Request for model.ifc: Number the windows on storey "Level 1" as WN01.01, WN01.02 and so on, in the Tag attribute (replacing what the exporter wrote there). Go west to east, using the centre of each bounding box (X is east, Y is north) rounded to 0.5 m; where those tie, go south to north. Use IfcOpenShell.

First a look at what the model holds.

```python
import ifcopenshell
import ifcopenshell.util.element
import ifcopenshell.util.placement

model = ifcopenshell.open("model.ifc")
print(model.schema)
storey = next(s for s in model.by_type("IfcBuildingStorey") if s.Name == "Level 1")
windows = [e for e in ifcopenshell.util.element.get_decomposition(storey) if e.is_a("IfcWindow")]
for e in sorted(windows, key=lambda e: e.id()):
    origin = ifcopenshell.util.placement.get_local_placement(e.ObjectPlacement)[:3, 3]
    print(e.id(), e.Tag, e.Name, origin.round(2) + 0.0, sep=" | ")
```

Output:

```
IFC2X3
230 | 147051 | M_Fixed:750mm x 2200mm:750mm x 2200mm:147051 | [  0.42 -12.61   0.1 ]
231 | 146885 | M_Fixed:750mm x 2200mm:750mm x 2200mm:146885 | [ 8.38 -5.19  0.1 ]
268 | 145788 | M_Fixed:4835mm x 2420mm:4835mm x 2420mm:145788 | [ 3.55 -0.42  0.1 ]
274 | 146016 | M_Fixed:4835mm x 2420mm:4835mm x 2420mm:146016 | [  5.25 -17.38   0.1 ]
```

```python
import ifcopenshell
import ifcopenshell.geom
import ifcopenshell.util.element
import ifcopenshell.util.shape

model = ifcopenshell.open("model.ifc")
settings = ifcopenshell.geom.settings()
settings.set("use-world-coords", True)


def centre(element):
    shape = ifcopenshell.geom.create_shape(settings, element)
    return ifcopenshell.util.shape.get_bbox_centroid(shape.geometry)


storey = next(s for s in model.by_type("IfcBuildingStorey") if s.Name == "Level 1")
windows = [e for e in ifcopenshell.util.element.get_decomposition(storey) if e.is_a("IfcWindow")]

# Insertion points can sit at a corner or the storey origin, so sort by the geometry (in metres).
centres = {e: centre(e) for e in windows}
windows.sort(key=lambda e: (round(centres[e][0] / 0.5), centres[e][1]))

for i, e in enumerate(windows, start=1):
    number = f"WN01.{i:02d}"
    e.Tag = number
    print(e.id(), number)

model.write("model_edited.ifc")
```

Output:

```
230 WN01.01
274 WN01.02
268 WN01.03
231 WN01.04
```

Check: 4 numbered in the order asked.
